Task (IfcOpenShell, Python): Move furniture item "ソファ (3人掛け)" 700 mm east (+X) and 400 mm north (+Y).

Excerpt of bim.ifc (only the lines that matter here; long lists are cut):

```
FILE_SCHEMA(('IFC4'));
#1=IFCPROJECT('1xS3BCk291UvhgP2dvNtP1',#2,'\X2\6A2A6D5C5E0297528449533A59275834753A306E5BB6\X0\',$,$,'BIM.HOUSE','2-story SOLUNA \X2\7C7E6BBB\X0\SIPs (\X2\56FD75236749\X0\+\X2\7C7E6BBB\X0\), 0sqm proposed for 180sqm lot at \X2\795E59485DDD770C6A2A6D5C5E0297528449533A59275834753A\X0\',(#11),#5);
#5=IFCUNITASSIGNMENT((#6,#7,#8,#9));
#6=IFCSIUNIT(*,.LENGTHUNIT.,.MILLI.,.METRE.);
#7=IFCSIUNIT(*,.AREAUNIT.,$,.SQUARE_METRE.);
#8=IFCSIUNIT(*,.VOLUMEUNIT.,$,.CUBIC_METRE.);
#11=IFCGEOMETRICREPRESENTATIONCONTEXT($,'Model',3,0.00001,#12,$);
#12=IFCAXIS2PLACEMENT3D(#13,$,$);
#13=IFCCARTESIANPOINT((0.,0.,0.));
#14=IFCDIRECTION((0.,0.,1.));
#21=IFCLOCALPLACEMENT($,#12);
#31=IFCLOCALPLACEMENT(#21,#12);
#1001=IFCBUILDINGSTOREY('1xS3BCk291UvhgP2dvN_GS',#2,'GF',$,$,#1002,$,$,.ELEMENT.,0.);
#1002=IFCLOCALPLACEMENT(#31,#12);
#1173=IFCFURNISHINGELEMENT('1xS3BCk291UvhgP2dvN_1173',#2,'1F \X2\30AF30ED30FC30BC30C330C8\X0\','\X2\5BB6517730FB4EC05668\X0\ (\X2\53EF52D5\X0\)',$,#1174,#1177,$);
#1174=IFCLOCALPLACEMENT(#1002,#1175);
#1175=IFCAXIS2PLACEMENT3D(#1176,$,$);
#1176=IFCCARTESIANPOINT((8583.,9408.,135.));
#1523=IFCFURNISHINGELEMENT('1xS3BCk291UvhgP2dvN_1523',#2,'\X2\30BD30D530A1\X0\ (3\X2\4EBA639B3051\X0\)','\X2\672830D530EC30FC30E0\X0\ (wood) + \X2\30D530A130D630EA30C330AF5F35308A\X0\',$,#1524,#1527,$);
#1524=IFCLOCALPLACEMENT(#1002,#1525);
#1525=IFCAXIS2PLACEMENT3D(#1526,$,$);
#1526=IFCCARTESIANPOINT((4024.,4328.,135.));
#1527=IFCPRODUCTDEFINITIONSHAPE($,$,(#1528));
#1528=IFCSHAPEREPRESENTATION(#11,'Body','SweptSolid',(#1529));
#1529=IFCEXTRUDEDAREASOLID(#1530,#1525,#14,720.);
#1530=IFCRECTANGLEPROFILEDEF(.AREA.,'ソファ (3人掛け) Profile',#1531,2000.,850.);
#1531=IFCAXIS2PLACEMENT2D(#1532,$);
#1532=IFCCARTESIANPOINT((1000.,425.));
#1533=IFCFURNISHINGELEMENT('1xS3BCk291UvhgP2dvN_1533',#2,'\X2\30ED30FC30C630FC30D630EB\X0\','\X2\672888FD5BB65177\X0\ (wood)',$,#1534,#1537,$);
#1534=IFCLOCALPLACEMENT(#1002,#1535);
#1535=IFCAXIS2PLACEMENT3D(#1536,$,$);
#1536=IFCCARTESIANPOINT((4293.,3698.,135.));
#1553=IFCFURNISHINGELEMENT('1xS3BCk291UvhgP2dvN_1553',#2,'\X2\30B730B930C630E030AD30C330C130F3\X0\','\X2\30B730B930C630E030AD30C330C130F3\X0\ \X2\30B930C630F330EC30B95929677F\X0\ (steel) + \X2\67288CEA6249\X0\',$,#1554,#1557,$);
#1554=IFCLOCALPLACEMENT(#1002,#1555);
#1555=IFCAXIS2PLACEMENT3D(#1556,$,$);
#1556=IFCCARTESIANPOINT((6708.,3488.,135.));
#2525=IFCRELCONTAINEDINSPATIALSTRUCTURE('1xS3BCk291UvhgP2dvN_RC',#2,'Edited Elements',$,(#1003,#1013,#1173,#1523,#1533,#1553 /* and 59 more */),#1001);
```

```python
import ifcopenshell
import ifcopenshell.api.geometry
import ifcopenshell.util.placement
import ifcopenshell.util.unit

model = ifcopenshell.open("bim.ifc")
unit_scale = ifcopenshell.util.unit.calculate_unit_scale(model)

item = model.by_guid("1xS3BCk291UvhgP2dvN_1523")
matrix = ifcopenshell.util.placement.get_local_placement(item.ObjectPlacement)
matrix[0, 3] += 0.7 / unit_scale
matrix[1, 3] += 0.4 / unit_scale
ifcopenshell.api.geometry.edit_object_placement(model, product=item, matrix=matrix, is_si=False)

print(ifcopenshell.util.placement.get_local_placement(item.ObjectPlacement).round(3) + 0.0)

model.write("bim_rev.ifc")
```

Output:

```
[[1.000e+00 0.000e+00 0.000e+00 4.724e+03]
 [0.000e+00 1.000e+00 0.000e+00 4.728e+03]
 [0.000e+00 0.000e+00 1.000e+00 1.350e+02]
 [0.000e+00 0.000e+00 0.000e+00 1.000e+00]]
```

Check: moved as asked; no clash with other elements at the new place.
